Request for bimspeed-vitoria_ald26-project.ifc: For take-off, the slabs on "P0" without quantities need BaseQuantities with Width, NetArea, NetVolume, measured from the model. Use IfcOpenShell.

First a look at what the model holds.

```python
import ifcopenshell
import ifcopenshell.util.element
import ifcopenshell.util.unit

model = ifcopenshell.open("bimspeed-vitoria_ald26-project.ifc")
print(model.schema)
for unit_type in ("LENGTHUNIT", "AREAUNIT", "VOLUMEUNIT"):
    print(unit_type, ifcopenshell.util.unit.calculate_unit_scale(model, unit_type))
storey = next(s for s in model.by_type("IfcBuildingStorey") if s.Name == "P0")
slabs = [e for e in ifcopenshell.util.element.get_decomposition(storey) if e.is_a("IfcSlab")]
for e in sorted(slabs, key=lambda e: e.id()):
    print(e.id(), e.is_a(), e.Name, list(ifcopenshell.util.element.get_psets(e, qtos_only=True)), sep=" | ")
```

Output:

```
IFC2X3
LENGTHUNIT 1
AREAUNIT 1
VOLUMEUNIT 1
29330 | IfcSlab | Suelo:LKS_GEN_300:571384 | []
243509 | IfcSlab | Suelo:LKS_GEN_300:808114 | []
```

```python
import ifcopenshell
import ifcopenshell.api.pset
import ifcopenshell.geom
import ifcopenshell.util.element
import ifcopenshell.util.shape
import ifcopenshell.util.unit

model = ifcopenshell.open("bimspeed-vitoria_ald26-project.ifc")
unit_scale = ifcopenshell.util.unit.calculate_unit_scale(model)
area_scale = ifcopenshell.util.unit.calculate_unit_scale(model, "AREAUNIT")
volume_scale = ifcopenshell.util.unit.calculate_unit_scale(model, "VOLUMEUNIT")
settings = ifcopenshell.geom.settings()

storey = next(s for s in model.by_type("IfcBuildingStorey") if s.Name == "P0")
slabs = [e for e in ifcopenshell.util.element.get_decomposition(storey) if e.is_a("IfcSlab")]

for e in sorted(slabs, key=lambda e: e.id()):
    if ifcopenshell.util.element.get_psets(e, qtos_only=True, should_inherit=False):
        continue
    # Geometry comes back in metres, in the element's own axes.
    shape = ifcopenshell.geom.create_shape(settings, e)
    values = {
        "Width": ifcopenshell.util.shape.get_z(shape.geometry) / unit_scale,
        "NetArea": ifcopenshell.util.shape.get_footprint_area(shape.geometry) / area_scale,
        "NetVolume": ifcopenshell.util.shape.get_volume(shape.geometry) / volume_scale,
    }
    qto = ifcopenshell.api.pset.add_qto(model, product=e, name="BaseQuantities")
    ifcopenshell.api.pset.edit_qto(model, qto=qto, properties=values)
    print(e.id(), {k: round(v, 3) for k, v in values.items()})

model.write("bimspeed-vitoria_ald26-project_edited.ifc")
```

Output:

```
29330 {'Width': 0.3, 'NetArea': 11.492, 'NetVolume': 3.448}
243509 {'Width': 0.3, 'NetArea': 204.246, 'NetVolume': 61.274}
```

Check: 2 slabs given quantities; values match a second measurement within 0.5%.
